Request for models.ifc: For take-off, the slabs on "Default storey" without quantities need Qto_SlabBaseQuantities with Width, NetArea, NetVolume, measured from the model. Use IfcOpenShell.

First a look at what the model holds.

```python
import ifcopenshell
import ifcopenshell.util.element
import ifcopenshell.util.unit

model = ifcopenshell.open("models.ifc")
print(model.schema)
for unit_type in ("LENGTHUNIT", "AREAUNIT", "VOLUMEUNIT"):
    print(unit_type, ifcopenshell.util.unit.calculate_unit_scale(model, unit_type))
storey = next(s for s in model.by_type("IfcBuildingStorey") if s.Name == "Default storey")
slabs = [e for e in ifcopenshell.util.element.get_decomposition(storey) if e.is_a("IfcSlab")]
for e in sorted(slabs, key=lambda e: e.id()):
    print(e.id(), e.is_a(), e.Name, list(ifcopenshell.util.element.get_psets(e, qtos_only=True)), sep=" | ")
```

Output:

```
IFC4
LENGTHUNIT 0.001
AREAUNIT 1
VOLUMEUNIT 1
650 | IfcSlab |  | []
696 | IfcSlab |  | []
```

```python
import ifcopenshell
import ifcopenshell.api.pset
import ifcopenshell.geom
import ifcopenshell.util.element
import ifcopenshell.util.shape
import ifcopenshell.util.unit

model = ifcopenshell.open("models.ifc")
unit_scale = ifcopenshell.util.unit.calculate_unit_scale(model)
area_scale = ifcopenshell.util.unit.calculate_unit_scale(model, "AREAUNIT")
volume_scale = ifcopenshell.util.unit.calculate_unit_scale(model, "VOLUMEUNIT")
settings = ifcopenshell.geom.settings()

storey = next(s for s in model.by_type("IfcBuildingStorey") if s.Name == "Default storey")
slabs = [e for e in ifcopenshell.util.element.get_decomposition(storey) if e.is_a("IfcSlab")]

for e in sorted(slabs, key=lambda e: e.id()):
    if ifcopenshell.util.element.get_psets(e, qtos_only=True, should_inherit=False):
        continue
    # Geometry comes back in metres, in the element's own axes.
    shape = ifcopenshell.geom.create_shape(settings, e)
    values = {
        "Width": ifcopenshell.util.shape.get_z(shape.geometry) / unit_scale,
        "NetArea": ifcopenshell.util.shape.get_footprint_area(shape.geometry) / area_scale,
        "NetVolume": ifcopenshell.util.shape.get_volume(shape.geometry) / volume_scale,
    }
    qto = ifcopenshell.api.pset.add_qto(model, product=e, name="Qto_SlabBaseQuantities")
    ifcopenshell.api.pset.edit_qto(model, qto=qto, properties=values)
    print(e.id(), {k: round(v, 3) for k, v in values.items()})

model.write("models_updated.ifc")
```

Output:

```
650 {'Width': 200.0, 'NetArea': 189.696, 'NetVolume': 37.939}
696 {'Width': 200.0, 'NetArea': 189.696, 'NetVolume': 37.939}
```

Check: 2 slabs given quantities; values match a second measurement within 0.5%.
